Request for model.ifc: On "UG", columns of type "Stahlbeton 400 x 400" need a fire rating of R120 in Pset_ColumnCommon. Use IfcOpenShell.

First a look at what the model holds.

```python
import ifcopenshell
import ifcopenshell.util.element

model = ifcopenshell.open("model.ifc")
print(model.schema)
storey = next(s for s in model.by_type("IfcBuildingStorey") if s.Name == "UG")
columns = [e for e in ifcopenshell.util.element.get_decomposition(storey) if e.is_a("IfcColumn")]
seen = {}
for e in columns:
    element_type = ifcopenshell.util.element.get_type(e)
    key = (element_type.Name if element_type != e and element_type else None, ifcopenshell.util.element.get_pset(e, "Pset_ColumnCommon", "FireRating"))
    seen[key] = seen.get(key, 0) + 1
for (name, value), count in sorted(seen.items(), key=str):
    print(count, "x", name, "|", value)
```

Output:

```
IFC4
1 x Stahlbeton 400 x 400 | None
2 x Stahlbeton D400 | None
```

```python
import ifcopenshell
import ifcopenshell.api.pset
import ifcopenshell.util.element

model = ifcopenshell.open("model.ifc")

storey = next(s for s in model.by_type("IfcBuildingStorey") if s.Name == "UG")
columns = [e for e in ifcopenshell.util.element.get_decomposition(storey) if e.is_a("IfcColumn")]

count = 0
for e in columns:
    element_type = ifcopenshell.util.element.get_type(e)
    if element_type in (None, e) or element_type.Name != "Stahlbeton 400 x 400":
        continue
    # add_pset returns the element's existing set when there is one.
    pset = ifcopenshell.api.pset.add_pset(model, product=e, name="Pset_ColumnCommon")
    ifcopenshell.api.pset.edit_pset(model, pset=pset, properties={"FireRating": "R120"})
    count += 1

print(count, "columns updated")

model.write("model-out.ifc")
```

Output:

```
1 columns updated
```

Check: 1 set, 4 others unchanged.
